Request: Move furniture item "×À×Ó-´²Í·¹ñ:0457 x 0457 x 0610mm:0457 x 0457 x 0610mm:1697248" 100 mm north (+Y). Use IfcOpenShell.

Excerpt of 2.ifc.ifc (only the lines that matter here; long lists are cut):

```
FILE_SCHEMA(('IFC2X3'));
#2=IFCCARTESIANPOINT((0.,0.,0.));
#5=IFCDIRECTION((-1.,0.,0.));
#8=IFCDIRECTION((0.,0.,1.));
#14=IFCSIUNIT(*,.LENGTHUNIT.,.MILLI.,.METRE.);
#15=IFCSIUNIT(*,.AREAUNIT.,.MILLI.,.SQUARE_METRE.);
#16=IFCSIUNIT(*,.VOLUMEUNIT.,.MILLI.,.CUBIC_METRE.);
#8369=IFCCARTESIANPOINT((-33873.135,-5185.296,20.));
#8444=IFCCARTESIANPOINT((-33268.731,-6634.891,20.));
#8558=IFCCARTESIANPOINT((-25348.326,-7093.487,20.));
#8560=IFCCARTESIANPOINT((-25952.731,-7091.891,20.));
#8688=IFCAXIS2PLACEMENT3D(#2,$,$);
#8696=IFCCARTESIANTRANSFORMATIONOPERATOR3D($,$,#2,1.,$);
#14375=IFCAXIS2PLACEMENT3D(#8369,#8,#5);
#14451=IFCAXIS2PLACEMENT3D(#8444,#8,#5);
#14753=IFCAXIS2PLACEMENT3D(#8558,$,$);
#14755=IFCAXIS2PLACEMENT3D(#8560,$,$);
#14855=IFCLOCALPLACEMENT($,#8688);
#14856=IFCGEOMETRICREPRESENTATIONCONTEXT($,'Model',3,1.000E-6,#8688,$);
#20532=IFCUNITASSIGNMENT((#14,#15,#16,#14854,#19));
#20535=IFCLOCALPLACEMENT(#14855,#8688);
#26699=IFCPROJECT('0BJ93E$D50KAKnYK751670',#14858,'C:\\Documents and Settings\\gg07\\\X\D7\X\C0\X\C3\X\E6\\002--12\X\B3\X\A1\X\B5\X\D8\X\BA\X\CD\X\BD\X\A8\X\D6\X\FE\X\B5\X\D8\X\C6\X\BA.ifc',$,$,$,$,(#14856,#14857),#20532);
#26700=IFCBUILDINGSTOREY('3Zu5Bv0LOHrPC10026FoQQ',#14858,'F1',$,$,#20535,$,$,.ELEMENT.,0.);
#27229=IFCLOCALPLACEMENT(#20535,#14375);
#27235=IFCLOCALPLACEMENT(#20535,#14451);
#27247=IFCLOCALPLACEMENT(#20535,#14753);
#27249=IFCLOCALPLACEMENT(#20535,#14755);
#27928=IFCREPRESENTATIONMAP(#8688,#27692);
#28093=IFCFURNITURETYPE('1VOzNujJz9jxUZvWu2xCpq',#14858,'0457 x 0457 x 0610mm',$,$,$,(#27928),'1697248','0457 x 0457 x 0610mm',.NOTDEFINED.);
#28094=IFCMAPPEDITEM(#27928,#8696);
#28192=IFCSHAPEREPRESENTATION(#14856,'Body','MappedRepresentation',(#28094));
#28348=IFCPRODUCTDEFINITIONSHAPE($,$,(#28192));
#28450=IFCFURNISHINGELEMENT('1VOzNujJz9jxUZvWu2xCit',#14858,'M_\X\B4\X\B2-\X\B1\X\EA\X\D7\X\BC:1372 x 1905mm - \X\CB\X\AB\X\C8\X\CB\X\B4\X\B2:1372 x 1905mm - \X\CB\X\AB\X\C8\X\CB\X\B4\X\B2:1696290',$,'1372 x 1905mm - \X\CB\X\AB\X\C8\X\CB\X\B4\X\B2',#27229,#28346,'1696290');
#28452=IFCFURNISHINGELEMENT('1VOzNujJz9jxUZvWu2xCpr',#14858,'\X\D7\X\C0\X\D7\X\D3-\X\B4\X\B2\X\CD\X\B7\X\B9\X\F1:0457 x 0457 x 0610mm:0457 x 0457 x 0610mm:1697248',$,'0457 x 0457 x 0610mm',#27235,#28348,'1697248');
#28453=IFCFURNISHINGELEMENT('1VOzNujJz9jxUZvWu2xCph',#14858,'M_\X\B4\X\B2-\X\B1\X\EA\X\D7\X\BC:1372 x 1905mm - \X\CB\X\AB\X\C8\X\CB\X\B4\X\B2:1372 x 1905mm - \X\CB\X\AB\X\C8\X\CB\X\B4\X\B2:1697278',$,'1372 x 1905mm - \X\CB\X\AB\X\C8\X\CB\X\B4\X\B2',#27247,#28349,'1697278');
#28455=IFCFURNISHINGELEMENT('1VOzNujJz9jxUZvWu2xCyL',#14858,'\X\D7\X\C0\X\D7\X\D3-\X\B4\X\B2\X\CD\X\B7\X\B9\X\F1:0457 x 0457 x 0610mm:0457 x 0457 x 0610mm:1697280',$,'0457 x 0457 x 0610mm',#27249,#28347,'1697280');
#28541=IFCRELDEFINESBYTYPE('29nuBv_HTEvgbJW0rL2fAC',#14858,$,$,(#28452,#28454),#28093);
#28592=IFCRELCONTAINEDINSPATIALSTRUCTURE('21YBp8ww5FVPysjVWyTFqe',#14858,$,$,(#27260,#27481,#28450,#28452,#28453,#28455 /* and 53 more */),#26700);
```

```python
import ifcopenshell
import ifcopenshell.api.geometry
import ifcopenshell.util.placement

model = ifcopenshell.open("2.ifc.ifc")

item = model.by_guid("1VOzNujJz9jxUZvWu2xCpr")
matrix = ifcopenshell.util.placement.get_local_placement(item.ObjectPlacement)
matrix[1, 3] += 100.0
ifcopenshell.api.geometry.edit_object_placement(model, product=item, matrix=matrix, is_si=False)

print(ifcopenshell.util.placement.get_local_placement(item.ObjectPlacement).round(3) + 0.0)

model.write("2.ifc_edited.ifc")
```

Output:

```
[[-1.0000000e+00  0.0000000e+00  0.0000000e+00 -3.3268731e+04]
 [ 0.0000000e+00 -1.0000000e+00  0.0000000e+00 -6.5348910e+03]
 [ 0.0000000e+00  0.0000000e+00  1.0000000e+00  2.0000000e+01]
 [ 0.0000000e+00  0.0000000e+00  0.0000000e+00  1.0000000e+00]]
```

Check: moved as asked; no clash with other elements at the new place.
